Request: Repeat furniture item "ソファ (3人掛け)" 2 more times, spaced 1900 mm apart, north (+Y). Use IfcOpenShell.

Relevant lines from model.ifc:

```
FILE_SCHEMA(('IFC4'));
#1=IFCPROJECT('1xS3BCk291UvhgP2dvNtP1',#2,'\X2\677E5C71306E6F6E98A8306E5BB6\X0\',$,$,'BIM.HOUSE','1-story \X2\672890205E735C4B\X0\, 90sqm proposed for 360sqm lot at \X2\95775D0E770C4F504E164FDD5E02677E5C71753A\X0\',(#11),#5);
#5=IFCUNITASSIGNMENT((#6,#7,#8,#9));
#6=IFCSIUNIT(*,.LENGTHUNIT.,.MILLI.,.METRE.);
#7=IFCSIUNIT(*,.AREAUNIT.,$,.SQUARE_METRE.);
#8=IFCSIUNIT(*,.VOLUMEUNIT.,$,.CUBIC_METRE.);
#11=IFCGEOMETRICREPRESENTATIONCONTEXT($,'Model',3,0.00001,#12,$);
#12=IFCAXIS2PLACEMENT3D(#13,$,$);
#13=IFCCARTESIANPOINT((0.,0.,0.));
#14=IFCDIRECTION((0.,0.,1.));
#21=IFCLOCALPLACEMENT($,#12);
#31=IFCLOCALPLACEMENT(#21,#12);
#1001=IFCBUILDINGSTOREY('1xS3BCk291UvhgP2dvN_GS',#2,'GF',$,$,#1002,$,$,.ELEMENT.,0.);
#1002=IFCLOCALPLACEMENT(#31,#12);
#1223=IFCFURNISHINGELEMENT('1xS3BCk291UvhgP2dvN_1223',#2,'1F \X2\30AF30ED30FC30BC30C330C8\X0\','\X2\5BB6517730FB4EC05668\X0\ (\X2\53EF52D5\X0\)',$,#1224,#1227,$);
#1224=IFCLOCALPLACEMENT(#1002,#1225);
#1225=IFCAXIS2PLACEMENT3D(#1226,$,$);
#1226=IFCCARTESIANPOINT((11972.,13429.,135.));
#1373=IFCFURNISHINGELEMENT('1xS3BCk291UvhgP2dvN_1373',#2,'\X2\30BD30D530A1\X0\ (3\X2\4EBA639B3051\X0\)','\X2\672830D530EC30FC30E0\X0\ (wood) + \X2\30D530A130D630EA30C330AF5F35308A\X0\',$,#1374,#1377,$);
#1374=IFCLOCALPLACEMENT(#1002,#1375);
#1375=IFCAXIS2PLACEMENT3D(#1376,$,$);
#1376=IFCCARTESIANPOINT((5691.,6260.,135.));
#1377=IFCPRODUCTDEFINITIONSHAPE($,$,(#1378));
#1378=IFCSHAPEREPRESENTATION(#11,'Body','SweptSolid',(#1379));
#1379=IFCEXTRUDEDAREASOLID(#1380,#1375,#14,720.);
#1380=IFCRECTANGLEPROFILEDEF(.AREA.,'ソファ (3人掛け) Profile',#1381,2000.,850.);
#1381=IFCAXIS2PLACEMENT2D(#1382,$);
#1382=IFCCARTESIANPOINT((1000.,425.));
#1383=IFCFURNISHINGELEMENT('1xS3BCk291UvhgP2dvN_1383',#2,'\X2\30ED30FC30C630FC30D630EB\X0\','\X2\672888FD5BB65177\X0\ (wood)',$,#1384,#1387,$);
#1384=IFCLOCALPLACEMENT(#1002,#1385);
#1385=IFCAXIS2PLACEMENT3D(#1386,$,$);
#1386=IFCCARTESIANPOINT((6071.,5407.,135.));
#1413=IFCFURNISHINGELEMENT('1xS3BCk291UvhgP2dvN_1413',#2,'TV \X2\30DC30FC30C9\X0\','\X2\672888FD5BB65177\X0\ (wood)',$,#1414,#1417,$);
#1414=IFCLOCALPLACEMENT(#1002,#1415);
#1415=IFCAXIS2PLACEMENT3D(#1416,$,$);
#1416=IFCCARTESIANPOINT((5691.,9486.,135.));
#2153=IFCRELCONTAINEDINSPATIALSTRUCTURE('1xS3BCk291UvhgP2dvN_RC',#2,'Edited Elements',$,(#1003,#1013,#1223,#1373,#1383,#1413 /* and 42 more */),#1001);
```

```python
import numpy as np
import ifcopenshell
import ifcopenshell.api.geometry
import ifcopenshell.api.root
import ifcopenshell.util.element
import ifcopenshell.util.placement
import ifcopenshell.util.unit

model = ifcopenshell.open("model.ifc")
unit_scale = ifcopenshell.util.unit.calculate_unit_scale(model)


def reuse_history(source, copy):
    """copy_class also copies each property set's owner history, people and application; keep the originals."""
    for rel in copy.IsDefinedBy:
        if rel.is_a("IfcRelDefinesByProperties") and (history := rel.RelatingPropertyDefinition.OwnerHistory):
            rel.RelatingPropertyDefinition.OwnerHistory = source.OwnerHistory
            ifcopenshell.util.element.remove_deep2(model, history)


source = model.by_guid("1xS3BCk291UvhgP2dvN_1373")
base = ifcopenshell.util.placement.get_local_placement(source.ObjectPlacement)
step = np.array([0.0, 1.0, 0.0]) * 1.9 / unit_scale

for i in range(1, 3):
    copy = ifcopenshell.api.root.copy_class(model, product=source)
    copy.Representation = ifcopenshell.util.element.copy_deep(
        model, source.Representation, exclude=["IfcGeometricRepresentationContext", "IfcRepresentationMap"]
    )
    reuse_history(source, copy)
    matrix = base.copy()
    matrix[:3, 3] += i * step
    print("added at", matrix[:3, 3].round(3) + 0.0)
    ifcopenshell.api.geometry.edit_object_placement(model, product=copy, matrix=matrix, is_si=False)

model.write("model-out.ifc")
```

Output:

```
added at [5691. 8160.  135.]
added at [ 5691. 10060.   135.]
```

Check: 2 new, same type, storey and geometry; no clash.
